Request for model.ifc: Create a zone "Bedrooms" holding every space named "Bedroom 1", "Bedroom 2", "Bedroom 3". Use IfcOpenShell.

First a look at what the model holds.

```python
import ifcopenshell

model = ifcopenshell.open("model.ifc")
print(model.schema)
seen = {}
for space in model.by_type("IfcSpace"):
    seen[space.LongName] = seen.get(space.LongName, 0) + 1
for name, count in sorted(seen.items(), key=str):
    print(count, "x", name)
print("zones:", [z.Name for z in model.by_type("IfcZone")][:20])
```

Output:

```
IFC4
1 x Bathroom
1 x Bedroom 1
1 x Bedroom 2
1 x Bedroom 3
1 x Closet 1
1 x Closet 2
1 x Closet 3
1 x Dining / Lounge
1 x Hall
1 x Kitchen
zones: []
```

```python
import ifcopenshell
import ifcopenshell.api.group
import ifcopenshell.api.root

model = ifcopenshell.open("model.ifc")

names = {"Bedroom 1", "Bedroom 2", "Bedroom 3"}
spaces = [s for s in model.by_type("IfcSpace") if s.LongName in names]

zone = ifcopenshell.api.root.create_entity(model, ifc_class="IfcZone", name="Bedrooms")
ifcopenshell.api.group.assign_group(model, products=spaces, group=zone)
print(len(spaces), "spaces in", zone.Name)

model.write("model_updated.ifc")
```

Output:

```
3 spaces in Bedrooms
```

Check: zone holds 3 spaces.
